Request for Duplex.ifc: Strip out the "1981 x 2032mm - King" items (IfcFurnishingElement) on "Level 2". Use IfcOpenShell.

First a look at what the model holds.

```python
import ifcopenshell
import ifcopenshell.util.element

model = ifcopenshell.open("Duplex.ifc")
print(model.schema)
storey = next(s for s in model.by_type("IfcBuildingStorey") if s.Name == "Level 2")
furniture = [e for e in ifcopenshell.util.element.get_decomposition(storey) if e.is_a("IfcFurnishingElement")]
seen = {}
for e in furniture:
    element_type = ifcopenshell.util.element.get_type(e)
    name = element_type.Name if element_type not in (None, e) else None
    seen[name] = seen.get(name, 0) + 1
for name, count in sorted(seen.items(), key=str):
    print(count, "x", name)
```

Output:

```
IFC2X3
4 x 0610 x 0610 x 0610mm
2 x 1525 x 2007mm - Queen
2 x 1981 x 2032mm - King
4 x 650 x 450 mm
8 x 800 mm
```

```python
import ifcopenshell
import ifcopenshell.api.root
import ifcopenshell.util.element

model = ifcopenshell.open("Duplex.ifc")

storey = next(s for s in model.by_type("IfcBuildingStorey") if s.Name == "Level 2")
furniture = [e for e in ifcopenshell.util.element.get_decomposition(storey) if e.is_a("IfcFurnishingElement")]
targets = [e for e in furniture if (t := ifcopenshell.util.element.get_type(e)) not in (None, e) and t.Name == "1981 x 2032mm - King"]

for e in targets:
    ifcopenshell.api.root.remove_product(model, product=e)
print(len(targets), "removed")

model.write("Duplex_v2.ifc")
```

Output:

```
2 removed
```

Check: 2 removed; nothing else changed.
